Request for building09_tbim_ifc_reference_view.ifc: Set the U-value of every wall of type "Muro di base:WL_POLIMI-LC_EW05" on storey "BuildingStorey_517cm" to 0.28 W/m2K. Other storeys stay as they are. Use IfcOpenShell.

First a look at what the model holds.

```python
import ifcopenshell
import ifcopenshell.util.element

model = ifcopenshell.open("building09_tbim_ifc_reference_view.ifc")
print(model.schema)
storey = next(s for s in model.by_type("IfcBuildingStorey") if s.Name == "BuildingStorey_517cm")
walls = [e for e in ifcopenshell.util.element.get_decomposition(storey) if e.is_a("IfcWall")]
seen = {}
for e in walls:
    element_type = ifcopenshell.util.element.get_type(e)
    key = (element_type.Name if element_type != e and element_type else None, ifcopenshell.util.element.get_pset(e, "Pset_WallCommon", "ThermalTransmittance"))
    seen[key] = seen.get(key, 0) + 1
for (name, value), count in sorted(seen.items(), key=str):
    print(count, "x", name, "|", value)
```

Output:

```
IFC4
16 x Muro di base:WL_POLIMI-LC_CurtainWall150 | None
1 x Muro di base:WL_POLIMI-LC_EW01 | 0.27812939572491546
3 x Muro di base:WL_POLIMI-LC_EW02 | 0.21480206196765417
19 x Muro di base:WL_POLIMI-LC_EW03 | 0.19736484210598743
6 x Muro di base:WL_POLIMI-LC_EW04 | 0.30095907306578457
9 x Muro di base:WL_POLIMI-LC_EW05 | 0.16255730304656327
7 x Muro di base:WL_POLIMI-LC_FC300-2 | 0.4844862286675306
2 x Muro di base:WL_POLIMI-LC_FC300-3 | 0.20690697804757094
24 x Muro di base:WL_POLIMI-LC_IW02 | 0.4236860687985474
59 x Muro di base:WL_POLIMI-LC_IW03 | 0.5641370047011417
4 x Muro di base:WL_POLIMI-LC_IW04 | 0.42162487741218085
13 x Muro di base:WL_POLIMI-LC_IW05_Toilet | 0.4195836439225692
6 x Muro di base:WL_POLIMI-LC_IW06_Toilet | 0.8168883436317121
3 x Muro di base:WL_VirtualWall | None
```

```python
import ifcopenshell
import ifcopenshell.api.pset
import ifcopenshell.util.element

model = ifcopenshell.open("building09_tbim_ifc_reference_view.ifc")

storey = next(s for s in model.by_type("IfcBuildingStorey") if s.Name == "BuildingStorey_517cm")
walls = [e for e in ifcopenshell.util.element.get_decomposition(storey) if e.is_a("IfcWall")]

count = 0
for e in walls:
    element_type = ifcopenshell.util.element.get_type(e)
    if element_type in (None, e) or element_type.Name != "Muro di base:WL_POLIMI-LC_EW05":
        continue
    # add_pset returns the element's existing set when there is one.
    pset = ifcopenshell.api.pset.add_pset(model, product=e, name="Pset_WallCommon")
    ifcopenshell.api.pset.edit_pset(model, pset=pset, properties={"ThermalTransmittance": 0.28})
    count += 1

print(count, "walls updated")

model.write("building09_tbim_ifc_reference_view_v2.ifc")
```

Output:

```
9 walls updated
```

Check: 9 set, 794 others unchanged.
